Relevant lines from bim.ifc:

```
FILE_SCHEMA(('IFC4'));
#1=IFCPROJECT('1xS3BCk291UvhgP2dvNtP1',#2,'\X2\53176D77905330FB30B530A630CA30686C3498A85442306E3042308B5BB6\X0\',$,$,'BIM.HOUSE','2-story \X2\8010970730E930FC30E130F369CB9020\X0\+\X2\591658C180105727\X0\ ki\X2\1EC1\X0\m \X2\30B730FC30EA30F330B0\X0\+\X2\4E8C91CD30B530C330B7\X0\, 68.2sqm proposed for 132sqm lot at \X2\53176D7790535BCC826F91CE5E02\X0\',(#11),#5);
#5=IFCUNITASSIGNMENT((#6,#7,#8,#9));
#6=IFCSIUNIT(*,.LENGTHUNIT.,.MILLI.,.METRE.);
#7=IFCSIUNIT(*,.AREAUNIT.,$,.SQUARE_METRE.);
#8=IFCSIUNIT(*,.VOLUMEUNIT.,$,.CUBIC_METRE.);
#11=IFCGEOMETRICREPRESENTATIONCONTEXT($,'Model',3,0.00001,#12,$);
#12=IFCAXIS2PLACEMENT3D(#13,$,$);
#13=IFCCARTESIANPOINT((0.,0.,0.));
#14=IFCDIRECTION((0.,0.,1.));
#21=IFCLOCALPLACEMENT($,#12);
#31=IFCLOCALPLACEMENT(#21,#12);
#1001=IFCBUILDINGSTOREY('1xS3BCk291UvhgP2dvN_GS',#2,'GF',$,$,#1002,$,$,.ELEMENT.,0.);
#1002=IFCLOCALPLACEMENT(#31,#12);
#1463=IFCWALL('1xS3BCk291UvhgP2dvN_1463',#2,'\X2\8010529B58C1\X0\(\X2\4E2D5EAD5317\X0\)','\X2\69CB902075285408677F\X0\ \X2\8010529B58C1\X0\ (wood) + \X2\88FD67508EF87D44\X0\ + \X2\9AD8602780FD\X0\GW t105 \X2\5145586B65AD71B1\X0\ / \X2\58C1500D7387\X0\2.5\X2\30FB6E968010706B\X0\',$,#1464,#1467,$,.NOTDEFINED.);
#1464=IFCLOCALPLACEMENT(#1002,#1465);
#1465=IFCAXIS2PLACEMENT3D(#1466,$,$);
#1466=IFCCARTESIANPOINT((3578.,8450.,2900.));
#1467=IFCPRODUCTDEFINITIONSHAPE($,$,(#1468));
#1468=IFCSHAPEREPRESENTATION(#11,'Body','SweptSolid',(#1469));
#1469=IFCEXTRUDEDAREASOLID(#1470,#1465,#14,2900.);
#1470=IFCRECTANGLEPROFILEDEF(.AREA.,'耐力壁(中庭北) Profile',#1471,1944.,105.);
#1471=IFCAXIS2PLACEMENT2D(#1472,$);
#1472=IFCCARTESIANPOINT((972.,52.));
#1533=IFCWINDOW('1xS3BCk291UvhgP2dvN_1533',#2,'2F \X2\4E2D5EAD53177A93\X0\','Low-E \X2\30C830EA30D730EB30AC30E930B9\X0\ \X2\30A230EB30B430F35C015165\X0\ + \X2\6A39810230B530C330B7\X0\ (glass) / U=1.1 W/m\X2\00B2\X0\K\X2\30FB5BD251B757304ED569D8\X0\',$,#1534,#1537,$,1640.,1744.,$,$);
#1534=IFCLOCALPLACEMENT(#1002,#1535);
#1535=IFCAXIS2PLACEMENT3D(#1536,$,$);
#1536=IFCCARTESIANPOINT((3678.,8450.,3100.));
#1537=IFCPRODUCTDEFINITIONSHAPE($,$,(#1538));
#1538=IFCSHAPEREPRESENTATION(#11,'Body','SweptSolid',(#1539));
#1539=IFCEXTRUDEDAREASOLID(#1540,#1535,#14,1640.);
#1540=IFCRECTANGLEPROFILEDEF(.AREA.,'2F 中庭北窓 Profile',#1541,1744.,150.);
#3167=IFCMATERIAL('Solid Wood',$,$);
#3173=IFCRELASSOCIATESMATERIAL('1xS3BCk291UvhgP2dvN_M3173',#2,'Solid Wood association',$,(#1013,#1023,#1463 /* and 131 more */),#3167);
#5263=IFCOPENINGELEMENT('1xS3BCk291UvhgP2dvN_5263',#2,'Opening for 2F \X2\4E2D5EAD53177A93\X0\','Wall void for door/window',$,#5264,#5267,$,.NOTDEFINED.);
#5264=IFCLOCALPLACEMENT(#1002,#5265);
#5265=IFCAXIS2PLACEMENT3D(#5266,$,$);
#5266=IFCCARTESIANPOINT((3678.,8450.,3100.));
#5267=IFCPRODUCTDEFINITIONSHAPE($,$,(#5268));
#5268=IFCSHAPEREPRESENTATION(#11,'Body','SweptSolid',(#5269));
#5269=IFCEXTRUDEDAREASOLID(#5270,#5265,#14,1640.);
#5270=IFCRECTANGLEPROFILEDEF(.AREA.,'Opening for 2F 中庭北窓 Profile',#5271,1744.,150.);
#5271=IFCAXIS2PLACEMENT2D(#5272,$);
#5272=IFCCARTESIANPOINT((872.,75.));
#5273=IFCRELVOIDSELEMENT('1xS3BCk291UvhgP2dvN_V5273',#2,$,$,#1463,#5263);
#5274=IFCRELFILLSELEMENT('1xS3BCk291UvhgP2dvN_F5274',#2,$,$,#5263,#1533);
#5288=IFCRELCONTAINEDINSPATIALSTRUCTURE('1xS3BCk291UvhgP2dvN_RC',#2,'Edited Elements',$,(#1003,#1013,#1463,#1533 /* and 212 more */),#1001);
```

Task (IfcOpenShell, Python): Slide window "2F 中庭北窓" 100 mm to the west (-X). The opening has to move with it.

```python
import ifcopenshell
import ifcopenshell.api.geometry
import ifcopenshell.util.placement
import ifcopenshell.util.unit

model = ifcopenshell.open("bim.ifc")
unit_scale = ifcopenshell.util.unit.calculate_unit_scale(model)

window = model.by_id(1533)
opening = window.FillsVoids[0].RelatingOpeningElement
wall = opening.VoidsElements[0].RelatingBuildingElement

wall_matrix = ifcopenshell.util.placement.get_local_placement(wall.ObjectPlacement)
shift = wall_matrix[:3, 0] * -0.1 / unit_scale
before = ifcopenshell.util.placement.get_local_placement(window.ObjectPlacement)[:3, 3].copy()

# The window is not placed relative to its opening, so move both.
for product in (opening, window):
    matrix = ifcopenshell.util.placement.get_local_placement(product.ObjectPlacement)
    matrix[:3, 3] += shift
    ifcopenshell.api.geometry.edit_object_placement(model, product=product, matrix=matrix, is_si=False)

after = ifcopenshell.util.placement.get_local_placement(window.ObjectPlacement)[:3, 3]
print("window moved by", (after - before).round(3) + 0.0)

model.write("bim_rev.ifc")
```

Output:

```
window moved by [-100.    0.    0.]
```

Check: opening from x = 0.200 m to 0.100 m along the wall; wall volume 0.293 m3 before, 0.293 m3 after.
